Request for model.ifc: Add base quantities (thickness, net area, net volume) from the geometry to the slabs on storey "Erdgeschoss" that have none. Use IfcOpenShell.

First a look at what the model holds.

```python
import ifcopenshell
import ifcopenshell.util.element
import ifcopenshell.util.unit

model = ifcopenshell.open("model.ifc")
print(model.schema)
for unit_type in ("LENGTHUNIT", "AREAUNIT", "VOLUMEUNIT"):
    print(unit_type, ifcopenshell.util.unit.calculate_unit_scale(model, unit_type))
storey = next(s for s in model.by_type("IfcBuildingStorey") if s.Name == "Erdgeschoss")
slabs = [e for e in ifcopenshell.util.element.get_decomposition(storey) if e.is_a("IfcSlab")]
for e in sorted(slabs, key=lambda e: e.id()):
    print(e.id(), e.is_a(), e.Name, list(ifcopenshell.util.element.get_psets(e, qtos_only=True)), sep=" | ")
```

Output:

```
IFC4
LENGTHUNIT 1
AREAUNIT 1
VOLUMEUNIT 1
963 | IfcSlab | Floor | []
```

```python
import ifcopenshell
import ifcopenshell.api.pset
import ifcopenshell.geom
import ifcopenshell.util.element
import ifcopenshell.util.shape
import ifcopenshell.util.unit

model = ifcopenshell.open("model.ifc")
unit_scale = ifcopenshell.util.unit.calculate_unit_scale(model)
area_scale = ifcopenshell.util.unit.calculate_unit_scale(model, "AREAUNIT")
volume_scale = ifcopenshell.util.unit.calculate_unit_scale(model, "VOLUMEUNIT")
settings = ifcopenshell.geom.settings()

storey = next(s for s in model.by_type("IfcBuildingStorey") if s.Name == "Erdgeschoss")
slabs = [e for e in ifcopenshell.util.element.get_decomposition(storey) if e.is_a("IfcSlab")]

for e in sorted(slabs, key=lambda e: e.id()):
    if ifcopenshell.util.element.get_psets(e, qtos_only=True, should_inherit=False):
        continue
    # Geometry comes back in metres, in the element's own axes.
    shape = ifcopenshell.geom.create_shape(settings, e)
    values = {
        "Width": ifcopenshell.util.shape.get_z(shape.geometry) / unit_scale,
        "NetArea": ifcopenshell.util.shape.get_footprint_area(shape.geometry) / area_scale,
        "NetVolume": ifcopenshell.util.shape.get_volume(shape.geometry) / volume_scale,
    }
    qto = ifcopenshell.api.pset.add_qto(model, product=e, name="Qto_SlabBaseQuantities")
    ifcopenshell.api.pset.edit_qto(model, qto=qto, properties=values)
    print(e.id(), {k: round(v, 3) for k, v in values.items()})

model.write("model_edited.ifc")
```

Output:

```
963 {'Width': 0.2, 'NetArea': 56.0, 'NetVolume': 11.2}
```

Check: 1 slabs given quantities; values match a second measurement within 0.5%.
